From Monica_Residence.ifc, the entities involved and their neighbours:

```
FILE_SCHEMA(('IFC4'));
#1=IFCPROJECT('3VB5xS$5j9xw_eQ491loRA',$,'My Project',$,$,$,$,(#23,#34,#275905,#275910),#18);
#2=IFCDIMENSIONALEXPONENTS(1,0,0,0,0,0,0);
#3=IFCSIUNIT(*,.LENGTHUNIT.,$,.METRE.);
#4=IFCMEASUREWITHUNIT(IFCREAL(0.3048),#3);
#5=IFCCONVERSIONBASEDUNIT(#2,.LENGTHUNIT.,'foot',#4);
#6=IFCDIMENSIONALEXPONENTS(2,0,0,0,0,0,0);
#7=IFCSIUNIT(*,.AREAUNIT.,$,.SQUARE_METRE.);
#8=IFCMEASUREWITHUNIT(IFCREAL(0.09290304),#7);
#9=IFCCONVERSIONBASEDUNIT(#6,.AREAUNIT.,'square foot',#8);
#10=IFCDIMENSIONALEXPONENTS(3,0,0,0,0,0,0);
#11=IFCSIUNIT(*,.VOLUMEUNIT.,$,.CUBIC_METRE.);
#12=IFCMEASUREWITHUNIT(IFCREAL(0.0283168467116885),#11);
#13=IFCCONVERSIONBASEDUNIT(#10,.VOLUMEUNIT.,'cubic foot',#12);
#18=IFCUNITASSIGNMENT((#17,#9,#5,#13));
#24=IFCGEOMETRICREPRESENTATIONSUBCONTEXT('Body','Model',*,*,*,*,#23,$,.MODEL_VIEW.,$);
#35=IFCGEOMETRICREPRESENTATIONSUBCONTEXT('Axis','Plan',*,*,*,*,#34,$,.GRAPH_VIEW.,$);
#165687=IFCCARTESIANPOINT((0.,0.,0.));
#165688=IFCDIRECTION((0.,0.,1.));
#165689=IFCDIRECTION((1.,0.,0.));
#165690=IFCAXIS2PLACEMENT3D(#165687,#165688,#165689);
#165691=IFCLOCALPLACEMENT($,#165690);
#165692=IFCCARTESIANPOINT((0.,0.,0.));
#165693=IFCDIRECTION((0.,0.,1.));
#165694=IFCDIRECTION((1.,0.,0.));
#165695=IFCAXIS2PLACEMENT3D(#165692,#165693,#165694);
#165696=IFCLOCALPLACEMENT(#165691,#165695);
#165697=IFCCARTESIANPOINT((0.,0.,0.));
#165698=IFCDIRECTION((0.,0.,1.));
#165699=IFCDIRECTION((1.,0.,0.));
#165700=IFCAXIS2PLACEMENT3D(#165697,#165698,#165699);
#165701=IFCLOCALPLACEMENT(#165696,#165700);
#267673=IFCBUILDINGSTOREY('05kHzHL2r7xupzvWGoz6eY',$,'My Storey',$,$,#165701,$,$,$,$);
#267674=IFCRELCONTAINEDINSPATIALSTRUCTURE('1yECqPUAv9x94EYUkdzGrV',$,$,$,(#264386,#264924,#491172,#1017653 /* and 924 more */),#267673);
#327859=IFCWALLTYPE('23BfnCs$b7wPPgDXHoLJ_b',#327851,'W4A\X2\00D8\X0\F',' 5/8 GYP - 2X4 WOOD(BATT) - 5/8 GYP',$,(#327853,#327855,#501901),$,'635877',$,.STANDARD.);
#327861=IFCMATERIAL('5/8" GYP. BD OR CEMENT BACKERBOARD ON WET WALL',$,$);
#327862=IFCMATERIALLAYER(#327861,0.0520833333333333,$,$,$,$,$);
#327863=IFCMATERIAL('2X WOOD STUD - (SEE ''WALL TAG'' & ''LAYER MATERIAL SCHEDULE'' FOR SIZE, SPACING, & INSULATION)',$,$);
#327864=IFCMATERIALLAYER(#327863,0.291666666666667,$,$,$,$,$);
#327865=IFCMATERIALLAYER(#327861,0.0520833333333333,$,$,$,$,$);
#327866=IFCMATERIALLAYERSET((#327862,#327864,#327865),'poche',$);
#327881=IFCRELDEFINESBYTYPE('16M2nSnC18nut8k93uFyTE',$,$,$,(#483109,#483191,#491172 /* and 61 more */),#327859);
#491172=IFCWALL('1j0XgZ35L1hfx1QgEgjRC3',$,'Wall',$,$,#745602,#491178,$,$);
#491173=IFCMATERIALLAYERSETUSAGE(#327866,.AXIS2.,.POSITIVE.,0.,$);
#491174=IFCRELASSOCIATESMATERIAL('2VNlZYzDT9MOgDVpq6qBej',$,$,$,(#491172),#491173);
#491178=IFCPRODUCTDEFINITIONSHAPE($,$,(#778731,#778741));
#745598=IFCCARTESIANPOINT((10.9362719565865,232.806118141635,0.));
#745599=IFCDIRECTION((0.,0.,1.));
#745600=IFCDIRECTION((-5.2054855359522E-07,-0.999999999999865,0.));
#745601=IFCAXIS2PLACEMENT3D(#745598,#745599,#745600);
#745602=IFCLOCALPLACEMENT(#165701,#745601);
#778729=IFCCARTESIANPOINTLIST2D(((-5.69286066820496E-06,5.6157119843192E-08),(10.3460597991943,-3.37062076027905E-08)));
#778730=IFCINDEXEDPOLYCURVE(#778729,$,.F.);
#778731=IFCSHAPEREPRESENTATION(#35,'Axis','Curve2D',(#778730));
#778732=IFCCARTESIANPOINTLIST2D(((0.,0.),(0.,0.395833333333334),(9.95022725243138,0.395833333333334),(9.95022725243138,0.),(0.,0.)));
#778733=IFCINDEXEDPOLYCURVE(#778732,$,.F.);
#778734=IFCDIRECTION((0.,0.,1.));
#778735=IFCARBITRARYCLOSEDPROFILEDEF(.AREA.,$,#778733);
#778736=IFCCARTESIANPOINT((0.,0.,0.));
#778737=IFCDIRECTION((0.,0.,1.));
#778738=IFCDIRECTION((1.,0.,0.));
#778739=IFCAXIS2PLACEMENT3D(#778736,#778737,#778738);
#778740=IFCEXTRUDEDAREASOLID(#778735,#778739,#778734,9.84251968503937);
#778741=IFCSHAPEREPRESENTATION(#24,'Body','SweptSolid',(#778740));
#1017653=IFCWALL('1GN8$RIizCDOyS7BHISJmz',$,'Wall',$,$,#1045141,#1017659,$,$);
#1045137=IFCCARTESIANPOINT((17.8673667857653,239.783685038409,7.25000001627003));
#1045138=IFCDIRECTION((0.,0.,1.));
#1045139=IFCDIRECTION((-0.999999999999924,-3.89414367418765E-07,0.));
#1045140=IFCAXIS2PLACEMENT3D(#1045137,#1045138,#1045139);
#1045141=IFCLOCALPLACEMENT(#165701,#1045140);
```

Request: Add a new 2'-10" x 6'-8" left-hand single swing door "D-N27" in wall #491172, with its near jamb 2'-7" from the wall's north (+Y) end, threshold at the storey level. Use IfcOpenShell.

```python
import numpy as np
import ifcopenshell
import ifcopenshell.api.feature
import ifcopenshell.api.geometry
import ifcopenshell.api.root
import ifcopenshell.api.spatial
import ifcopenshell.geom
import ifcopenshell.util.element
import ifcopenshell.util.placement
import ifcopenshell.util.representation
import ifcopenshell.util.shape
import ifcopenshell.util.unit

model = ifcopenshell.open("Monica_Residence.ifc")
unit_scale = ifcopenshell.util.unit.calculate_unit_scale(model)
settings = ifcopenshell.geom.settings()


def volume(element):
    """Net volume in cubic metres, openings subtracted."""
    shape = ifcopenshell.geom.create_shape(settings, element)
    return ifcopenshell.util.shape.get_volume(shape.geometry)


wall = model.by_guid("1j0XgZ35L1hfx1QgEgjRC3")
storey = ifcopenshell.util.element.get_container(wall, ifc_class="IfcBuildingStorey")
context = ifcopenshell.util.representation.get_context(model, "Model", "Body", "MODEL_VIEW")
before = volume(wall)

width, height, from_end, sill = 0.8636, 2.032, 0.7874, 0.0  # metres

# The wall runs along its own X axis, and the end named is its -X end.
wall_shape = ifcopenshell.geom.create_shape(settings, wall)
x, y, z = ifcopenshell.util.shape.get_vertices(wall_shape.geometry).T
start = x.min() + from_end
face, thickness = float(y.min()), float(y.max() - y.min())
wall_matrix = ifcopenshell.util.placement.get_local_placement(wall.ObjectPlacement)
level = ifcopenshell.util.placement.get_local_placement(storey.ObjectPlacement)[2, 3]


def in_wall(x, y):
    """Placement at x, y metres in the wall's axes, at sill height."""
    matrix = wall_matrix.copy()
    matrix[:, 3] = wall_matrix @ np.array([x / unit_scale, y / unit_scale, 0.0, 1.0])
    matrix[2, 3] = level + sill / unit_scale
    return matrix


# Opening: a box that overshoots both wall faces by 50 mm.
opening = ifcopenshell.api.root.create_entity(model, ifc_class="IfcOpeningElement", predefined_type="OPENING")
box = ifcopenshell.api.geometry.add_wall_representation(
    model, context=context, length=width, height=height, thickness=thickness + 0.1
)
ifcopenshell.api.geometry.assign_representation(model, product=opening, representation=box)
ifcopenshell.api.geometry.edit_object_placement(model, product=opening, matrix=in_wall(start, face - 0.05), is_si=False)
ifcopenshell.api.feature.add_feature(model, feature=opening, element=wall)

door = ifcopenshell.api.root.create_entity(model, ifc_class="IfcDoor", name="D-N27", predefined_type="DOOR")
door.OverallWidth, door.OverallHeight = width / unit_scale, height / unit_scale
door.OperationType = "SINGLE_SWING_LEFT"
body = ifcopenshell.api.geometry.add_door_representation(
    model,
    context=context,
    overall_width=door.OverallWidth,
    overall_height=door.OverallHeight,
    operation_type="SINGLE_SWING_LEFT",
    lining_properties={"LiningDepth": thickness / unit_scale, "ThresholdDepth": thickness / unit_scale},
)
ifcopenshell.api.geometry.assign_representation(model, product=door, representation=body)
ifcopenshell.api.spatial.assign_container(model, products=[door], relating_structure=storey)
ifcopenshell.api.feature.add_filling(model, opening=opening, element=door)

# The lining spans the wall, so the door starts at the wall face.
ifcopenshell.api.geometry.edit_object_placement(model, product=door, matrix=in_wall(start, face), is_si=False)

after = volume(wall)

print(f"wall volume {before:.3f} -> {after:.3f} m3")

model.write("Monica_Residence_edited.ifc")
```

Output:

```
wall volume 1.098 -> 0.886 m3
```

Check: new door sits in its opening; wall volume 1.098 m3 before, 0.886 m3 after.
